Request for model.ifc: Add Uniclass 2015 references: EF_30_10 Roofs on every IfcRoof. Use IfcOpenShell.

First a look at what the model holds.

```python
import ifcopenshell

model = ifcopenshell.open("model.ifc")
print(model.schema)
print("classifications:", [c.Name for c in model.by_type("IfcClassification")])
for ifc_class in ("IfcDoor", "IfcRoof", "IfcStair", "IfcWall", "IfcWindow"):
    print(ifc_class, len(model.by_type(ifc_class)))
```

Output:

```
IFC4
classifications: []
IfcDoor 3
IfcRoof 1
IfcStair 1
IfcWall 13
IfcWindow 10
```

```python
import ifcopenshell
import ifcopenshell.api.classification

model = ifcopenshell.open("model.ifc")

system = ifcopenshell.api.classification.add_classification(model, classification="Uniclass 2015")

codes = {
    "IfcRoof": ("EF_30_10", "Roofs"),
}
for ifc_class, (code, name) in codes.items():
    products = model.by_type(ifc_class)
    ifcopenshell.api.classification.add_reference(
        model, products=products, classification=system, identification=code, name=name
    )
    print(code, len(products))

model.write("model-out.ifc")
```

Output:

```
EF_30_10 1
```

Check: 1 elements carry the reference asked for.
